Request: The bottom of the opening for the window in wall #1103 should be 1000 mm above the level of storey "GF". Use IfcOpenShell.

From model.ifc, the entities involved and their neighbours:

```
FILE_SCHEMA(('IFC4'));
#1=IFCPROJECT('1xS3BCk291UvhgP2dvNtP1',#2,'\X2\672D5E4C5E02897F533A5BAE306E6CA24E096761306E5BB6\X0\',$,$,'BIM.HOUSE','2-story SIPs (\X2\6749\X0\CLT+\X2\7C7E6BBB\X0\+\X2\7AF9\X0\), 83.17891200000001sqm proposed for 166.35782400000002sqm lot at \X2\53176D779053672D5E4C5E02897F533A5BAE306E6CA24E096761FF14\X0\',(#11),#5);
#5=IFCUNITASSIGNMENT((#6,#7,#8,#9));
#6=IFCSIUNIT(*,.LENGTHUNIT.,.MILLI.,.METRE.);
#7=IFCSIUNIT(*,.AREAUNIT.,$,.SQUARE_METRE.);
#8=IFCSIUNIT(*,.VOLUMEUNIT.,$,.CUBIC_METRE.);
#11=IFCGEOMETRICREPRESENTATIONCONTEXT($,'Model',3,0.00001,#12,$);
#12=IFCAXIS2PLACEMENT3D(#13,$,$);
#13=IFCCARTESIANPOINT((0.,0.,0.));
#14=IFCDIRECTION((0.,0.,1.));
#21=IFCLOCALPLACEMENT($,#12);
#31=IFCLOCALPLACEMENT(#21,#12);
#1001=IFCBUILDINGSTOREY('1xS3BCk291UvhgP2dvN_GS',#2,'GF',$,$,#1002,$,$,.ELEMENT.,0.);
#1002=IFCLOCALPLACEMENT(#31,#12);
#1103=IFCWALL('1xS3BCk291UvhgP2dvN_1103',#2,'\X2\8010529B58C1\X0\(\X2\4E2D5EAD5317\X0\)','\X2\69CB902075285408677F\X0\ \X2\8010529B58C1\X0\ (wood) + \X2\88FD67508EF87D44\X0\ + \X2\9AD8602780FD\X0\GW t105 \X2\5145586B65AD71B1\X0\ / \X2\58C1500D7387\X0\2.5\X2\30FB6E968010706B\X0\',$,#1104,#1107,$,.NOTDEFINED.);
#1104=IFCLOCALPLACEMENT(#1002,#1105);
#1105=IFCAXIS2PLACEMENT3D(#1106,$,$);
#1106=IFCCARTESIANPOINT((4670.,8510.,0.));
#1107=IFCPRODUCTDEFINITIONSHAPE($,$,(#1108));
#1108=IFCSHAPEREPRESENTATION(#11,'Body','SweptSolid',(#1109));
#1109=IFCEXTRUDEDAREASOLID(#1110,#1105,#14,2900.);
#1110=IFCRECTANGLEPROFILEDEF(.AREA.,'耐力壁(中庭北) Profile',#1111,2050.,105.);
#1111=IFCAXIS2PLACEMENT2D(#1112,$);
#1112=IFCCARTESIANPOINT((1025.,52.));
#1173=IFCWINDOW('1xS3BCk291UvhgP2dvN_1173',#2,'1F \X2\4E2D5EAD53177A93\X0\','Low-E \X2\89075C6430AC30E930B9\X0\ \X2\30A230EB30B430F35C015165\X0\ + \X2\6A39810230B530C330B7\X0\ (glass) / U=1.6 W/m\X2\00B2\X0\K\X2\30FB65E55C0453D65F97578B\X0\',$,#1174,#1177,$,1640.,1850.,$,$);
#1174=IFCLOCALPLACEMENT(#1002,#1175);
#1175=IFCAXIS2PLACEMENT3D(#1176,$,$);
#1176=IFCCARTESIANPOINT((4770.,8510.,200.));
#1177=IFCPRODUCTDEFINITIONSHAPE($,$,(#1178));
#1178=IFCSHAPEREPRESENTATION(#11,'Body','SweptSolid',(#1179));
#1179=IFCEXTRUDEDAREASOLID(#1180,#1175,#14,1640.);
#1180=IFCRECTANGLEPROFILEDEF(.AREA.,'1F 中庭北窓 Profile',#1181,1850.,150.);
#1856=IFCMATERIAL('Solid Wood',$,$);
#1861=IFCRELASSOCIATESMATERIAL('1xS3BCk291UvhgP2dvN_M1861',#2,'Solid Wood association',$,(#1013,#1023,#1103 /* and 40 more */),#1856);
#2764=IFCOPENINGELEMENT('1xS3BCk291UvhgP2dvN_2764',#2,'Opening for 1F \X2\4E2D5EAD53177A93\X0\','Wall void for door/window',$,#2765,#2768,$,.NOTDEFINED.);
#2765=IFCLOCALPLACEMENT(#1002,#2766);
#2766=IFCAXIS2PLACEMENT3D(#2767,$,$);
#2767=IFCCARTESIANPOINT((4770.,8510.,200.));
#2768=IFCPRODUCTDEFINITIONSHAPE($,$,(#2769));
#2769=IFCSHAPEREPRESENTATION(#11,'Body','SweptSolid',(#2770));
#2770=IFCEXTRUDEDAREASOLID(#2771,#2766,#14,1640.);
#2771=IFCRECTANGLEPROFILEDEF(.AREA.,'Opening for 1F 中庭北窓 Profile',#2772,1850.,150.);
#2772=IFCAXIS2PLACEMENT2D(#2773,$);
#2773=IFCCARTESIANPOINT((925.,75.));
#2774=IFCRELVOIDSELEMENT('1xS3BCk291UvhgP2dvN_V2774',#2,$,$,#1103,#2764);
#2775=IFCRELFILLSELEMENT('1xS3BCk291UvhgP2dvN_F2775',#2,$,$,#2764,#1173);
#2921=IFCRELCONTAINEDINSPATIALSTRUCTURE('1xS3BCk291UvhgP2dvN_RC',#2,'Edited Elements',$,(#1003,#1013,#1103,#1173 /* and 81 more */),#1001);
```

```python
import numpy as np
import ifcopenshell
import ifcopenshell.api.geometry
import ifcopenshell.geom
import ifcopenshell.util.element
import ifcopenshell.util.placement
import ifcopenshell.util.shape
import ifcopenshell.util.unit

model = ifcopenshell.open("model.ifc")
unit_scale = ifcopenshell.util.unit.calculate_unit_scale(model)

window = model.by_guid("1xS3BCk291UvhgP2dvN_1173")
opening = window.FillsVoids[0].RelatingOpeningElement
storey = ifcopenshell.util.element.get_container(window, ifc_class="IfcBuildingStorey")
level = ifcopenshell.util.placement.get_local_placement(storey.ObjectPlacement)[2, 3]

# The opening's origin need not be at the sill, so measure its lowest point.
shape = ifcopenshell.geom.create_shape(ifcopenshell.geom.settings(), opening)
bottom = ifcopenshell.util.shape.get_shape_bottom_elevation(shape, shape.geometry) / unit_scale
dz = level + 1000.0 - bottom

shift = np.array([0.0, 0.0, dz])
# The window is not placed relative to its opening, so move both.
for product in (opening, window):
    matrix = ifcopenshell.util.placement.get_local_placement(product.ObjectPlacement)
    matrix[:3, 3] += shift
    ifcopenshell.api.geometry.edit_object_placement(model, product=product, matrix=matrix, is_si=False)

print(f"moved by {dz * unit_scale:+.3f} m")

model.write("model_edited.ifc")
```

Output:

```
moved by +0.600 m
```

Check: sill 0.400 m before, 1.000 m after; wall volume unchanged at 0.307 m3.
